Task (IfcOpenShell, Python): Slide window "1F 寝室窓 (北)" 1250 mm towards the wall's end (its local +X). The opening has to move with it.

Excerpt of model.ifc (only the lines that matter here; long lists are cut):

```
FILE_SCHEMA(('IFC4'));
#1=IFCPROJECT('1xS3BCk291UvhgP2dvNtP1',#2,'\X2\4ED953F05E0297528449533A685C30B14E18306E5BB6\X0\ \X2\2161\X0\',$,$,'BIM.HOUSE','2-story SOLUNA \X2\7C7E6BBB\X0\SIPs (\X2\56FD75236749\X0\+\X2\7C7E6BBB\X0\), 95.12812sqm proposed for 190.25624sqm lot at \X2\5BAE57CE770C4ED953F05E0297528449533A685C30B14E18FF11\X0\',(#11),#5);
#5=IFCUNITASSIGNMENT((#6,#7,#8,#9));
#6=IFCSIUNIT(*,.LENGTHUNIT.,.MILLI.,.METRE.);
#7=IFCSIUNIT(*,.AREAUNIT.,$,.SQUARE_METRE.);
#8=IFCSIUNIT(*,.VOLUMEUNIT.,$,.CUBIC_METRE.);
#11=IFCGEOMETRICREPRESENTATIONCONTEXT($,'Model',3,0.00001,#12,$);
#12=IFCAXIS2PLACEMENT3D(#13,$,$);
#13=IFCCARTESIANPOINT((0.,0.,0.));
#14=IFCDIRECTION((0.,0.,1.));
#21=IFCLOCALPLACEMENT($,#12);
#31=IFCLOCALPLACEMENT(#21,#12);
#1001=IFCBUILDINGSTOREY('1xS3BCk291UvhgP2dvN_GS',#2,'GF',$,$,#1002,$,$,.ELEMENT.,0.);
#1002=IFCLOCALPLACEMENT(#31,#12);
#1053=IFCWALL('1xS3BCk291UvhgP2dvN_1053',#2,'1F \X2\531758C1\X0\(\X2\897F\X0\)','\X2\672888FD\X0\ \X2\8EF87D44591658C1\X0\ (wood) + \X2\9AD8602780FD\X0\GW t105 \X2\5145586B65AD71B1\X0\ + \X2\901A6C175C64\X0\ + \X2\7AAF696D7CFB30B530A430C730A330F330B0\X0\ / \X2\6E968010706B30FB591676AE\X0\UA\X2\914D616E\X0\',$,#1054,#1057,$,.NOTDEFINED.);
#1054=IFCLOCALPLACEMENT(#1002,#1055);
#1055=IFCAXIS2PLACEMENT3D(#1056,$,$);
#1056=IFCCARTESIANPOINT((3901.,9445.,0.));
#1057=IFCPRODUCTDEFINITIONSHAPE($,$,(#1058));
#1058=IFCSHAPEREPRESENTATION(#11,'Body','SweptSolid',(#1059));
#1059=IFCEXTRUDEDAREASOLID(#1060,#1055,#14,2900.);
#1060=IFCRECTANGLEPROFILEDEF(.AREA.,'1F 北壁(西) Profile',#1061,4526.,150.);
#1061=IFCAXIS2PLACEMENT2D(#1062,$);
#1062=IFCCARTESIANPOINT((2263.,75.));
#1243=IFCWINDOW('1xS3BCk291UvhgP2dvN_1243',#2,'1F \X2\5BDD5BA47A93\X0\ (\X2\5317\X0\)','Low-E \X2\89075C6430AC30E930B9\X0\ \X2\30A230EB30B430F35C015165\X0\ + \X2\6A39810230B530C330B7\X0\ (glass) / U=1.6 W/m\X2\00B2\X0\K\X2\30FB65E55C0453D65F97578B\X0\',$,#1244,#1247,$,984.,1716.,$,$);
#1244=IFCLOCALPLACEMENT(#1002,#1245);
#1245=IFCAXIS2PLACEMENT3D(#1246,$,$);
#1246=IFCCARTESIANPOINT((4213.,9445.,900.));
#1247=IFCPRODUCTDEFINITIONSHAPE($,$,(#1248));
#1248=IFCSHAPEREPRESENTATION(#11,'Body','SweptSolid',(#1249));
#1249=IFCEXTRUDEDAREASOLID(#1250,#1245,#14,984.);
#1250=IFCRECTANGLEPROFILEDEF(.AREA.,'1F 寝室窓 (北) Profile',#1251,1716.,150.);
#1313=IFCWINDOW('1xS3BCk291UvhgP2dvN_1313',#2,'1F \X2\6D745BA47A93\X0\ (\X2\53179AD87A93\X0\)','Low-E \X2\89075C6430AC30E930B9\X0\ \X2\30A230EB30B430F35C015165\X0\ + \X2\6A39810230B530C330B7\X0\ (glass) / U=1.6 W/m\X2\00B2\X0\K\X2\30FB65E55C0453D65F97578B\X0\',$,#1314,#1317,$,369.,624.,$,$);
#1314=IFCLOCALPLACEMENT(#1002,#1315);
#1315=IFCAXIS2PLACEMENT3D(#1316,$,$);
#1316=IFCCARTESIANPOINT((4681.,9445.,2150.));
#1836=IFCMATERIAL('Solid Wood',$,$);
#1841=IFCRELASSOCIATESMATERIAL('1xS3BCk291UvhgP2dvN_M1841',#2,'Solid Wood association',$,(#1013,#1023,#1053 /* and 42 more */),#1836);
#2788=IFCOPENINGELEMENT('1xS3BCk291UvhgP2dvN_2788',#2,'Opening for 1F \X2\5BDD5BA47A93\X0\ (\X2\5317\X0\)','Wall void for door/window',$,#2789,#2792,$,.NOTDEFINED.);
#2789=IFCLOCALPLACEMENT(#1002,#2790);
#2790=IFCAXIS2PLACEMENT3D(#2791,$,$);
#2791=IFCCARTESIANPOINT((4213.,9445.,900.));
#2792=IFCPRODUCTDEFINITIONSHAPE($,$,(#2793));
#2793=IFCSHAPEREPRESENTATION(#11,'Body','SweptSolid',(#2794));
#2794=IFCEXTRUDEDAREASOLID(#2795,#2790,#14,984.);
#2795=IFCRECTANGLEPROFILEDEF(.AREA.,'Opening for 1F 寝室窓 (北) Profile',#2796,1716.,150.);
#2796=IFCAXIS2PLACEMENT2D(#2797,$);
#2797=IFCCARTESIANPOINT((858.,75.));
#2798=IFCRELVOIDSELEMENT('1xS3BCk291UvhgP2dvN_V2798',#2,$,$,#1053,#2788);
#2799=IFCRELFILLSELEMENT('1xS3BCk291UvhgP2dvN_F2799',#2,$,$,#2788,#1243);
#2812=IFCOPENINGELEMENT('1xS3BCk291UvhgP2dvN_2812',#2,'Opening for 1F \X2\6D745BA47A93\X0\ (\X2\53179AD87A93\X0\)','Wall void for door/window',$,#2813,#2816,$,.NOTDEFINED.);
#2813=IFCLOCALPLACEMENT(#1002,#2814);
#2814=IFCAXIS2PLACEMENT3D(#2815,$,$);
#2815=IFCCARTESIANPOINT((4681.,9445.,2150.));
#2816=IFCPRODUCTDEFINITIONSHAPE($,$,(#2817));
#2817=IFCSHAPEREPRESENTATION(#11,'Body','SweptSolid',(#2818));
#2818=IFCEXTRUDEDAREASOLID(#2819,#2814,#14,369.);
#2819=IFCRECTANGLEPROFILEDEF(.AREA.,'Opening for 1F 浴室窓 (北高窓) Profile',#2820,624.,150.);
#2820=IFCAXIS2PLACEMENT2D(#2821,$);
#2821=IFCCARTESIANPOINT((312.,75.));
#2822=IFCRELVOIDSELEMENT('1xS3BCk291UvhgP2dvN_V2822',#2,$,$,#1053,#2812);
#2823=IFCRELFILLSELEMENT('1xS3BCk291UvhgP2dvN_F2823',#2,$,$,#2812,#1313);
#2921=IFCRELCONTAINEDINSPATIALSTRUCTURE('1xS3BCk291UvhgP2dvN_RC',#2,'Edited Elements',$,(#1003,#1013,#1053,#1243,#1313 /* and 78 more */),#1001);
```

```python
import ifcopenshell
import ifcopenshell.api.geometry
import ifcopenshell.util.placement

model = ifcopenshell.open("model.ifc")

window = model.by_id(1243)
opening = window.FillsVoids[0].RelatingOpeningElement
wall = opening.VoidsElements[0].RelatingBuildingElement

wall_matrix = ifcopenshell.util.placement.get_local_placement(wall.ObjectPlacement)
shift = wall_matrix[:3, 0] * 1250.0
before = ifcopenshell.util.placement.get_local_placement(window.ObjectPlacement)[:3, 3].copy()

# The window is not placed relative to its opening, so move both.
for product in (opening, window):
    matrix = ifcopenshell.util.placement.get_local_placement(product.ObjectPlacement)
    matrix[:3, 3] += shift
    ifcopenshell.api.geometry.edit_object_placement(model, product=product, matrix=matrix, is_si=False)

after = ifcopenshell.util.placement.get_local_placement(window.ObjectPlacement)[:3, 3]
print("window moved by", (after - before).round(3) + 0.0)

model.write("model_edited.ifc")
```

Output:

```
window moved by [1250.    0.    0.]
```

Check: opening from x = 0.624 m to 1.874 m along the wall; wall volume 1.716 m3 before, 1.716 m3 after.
